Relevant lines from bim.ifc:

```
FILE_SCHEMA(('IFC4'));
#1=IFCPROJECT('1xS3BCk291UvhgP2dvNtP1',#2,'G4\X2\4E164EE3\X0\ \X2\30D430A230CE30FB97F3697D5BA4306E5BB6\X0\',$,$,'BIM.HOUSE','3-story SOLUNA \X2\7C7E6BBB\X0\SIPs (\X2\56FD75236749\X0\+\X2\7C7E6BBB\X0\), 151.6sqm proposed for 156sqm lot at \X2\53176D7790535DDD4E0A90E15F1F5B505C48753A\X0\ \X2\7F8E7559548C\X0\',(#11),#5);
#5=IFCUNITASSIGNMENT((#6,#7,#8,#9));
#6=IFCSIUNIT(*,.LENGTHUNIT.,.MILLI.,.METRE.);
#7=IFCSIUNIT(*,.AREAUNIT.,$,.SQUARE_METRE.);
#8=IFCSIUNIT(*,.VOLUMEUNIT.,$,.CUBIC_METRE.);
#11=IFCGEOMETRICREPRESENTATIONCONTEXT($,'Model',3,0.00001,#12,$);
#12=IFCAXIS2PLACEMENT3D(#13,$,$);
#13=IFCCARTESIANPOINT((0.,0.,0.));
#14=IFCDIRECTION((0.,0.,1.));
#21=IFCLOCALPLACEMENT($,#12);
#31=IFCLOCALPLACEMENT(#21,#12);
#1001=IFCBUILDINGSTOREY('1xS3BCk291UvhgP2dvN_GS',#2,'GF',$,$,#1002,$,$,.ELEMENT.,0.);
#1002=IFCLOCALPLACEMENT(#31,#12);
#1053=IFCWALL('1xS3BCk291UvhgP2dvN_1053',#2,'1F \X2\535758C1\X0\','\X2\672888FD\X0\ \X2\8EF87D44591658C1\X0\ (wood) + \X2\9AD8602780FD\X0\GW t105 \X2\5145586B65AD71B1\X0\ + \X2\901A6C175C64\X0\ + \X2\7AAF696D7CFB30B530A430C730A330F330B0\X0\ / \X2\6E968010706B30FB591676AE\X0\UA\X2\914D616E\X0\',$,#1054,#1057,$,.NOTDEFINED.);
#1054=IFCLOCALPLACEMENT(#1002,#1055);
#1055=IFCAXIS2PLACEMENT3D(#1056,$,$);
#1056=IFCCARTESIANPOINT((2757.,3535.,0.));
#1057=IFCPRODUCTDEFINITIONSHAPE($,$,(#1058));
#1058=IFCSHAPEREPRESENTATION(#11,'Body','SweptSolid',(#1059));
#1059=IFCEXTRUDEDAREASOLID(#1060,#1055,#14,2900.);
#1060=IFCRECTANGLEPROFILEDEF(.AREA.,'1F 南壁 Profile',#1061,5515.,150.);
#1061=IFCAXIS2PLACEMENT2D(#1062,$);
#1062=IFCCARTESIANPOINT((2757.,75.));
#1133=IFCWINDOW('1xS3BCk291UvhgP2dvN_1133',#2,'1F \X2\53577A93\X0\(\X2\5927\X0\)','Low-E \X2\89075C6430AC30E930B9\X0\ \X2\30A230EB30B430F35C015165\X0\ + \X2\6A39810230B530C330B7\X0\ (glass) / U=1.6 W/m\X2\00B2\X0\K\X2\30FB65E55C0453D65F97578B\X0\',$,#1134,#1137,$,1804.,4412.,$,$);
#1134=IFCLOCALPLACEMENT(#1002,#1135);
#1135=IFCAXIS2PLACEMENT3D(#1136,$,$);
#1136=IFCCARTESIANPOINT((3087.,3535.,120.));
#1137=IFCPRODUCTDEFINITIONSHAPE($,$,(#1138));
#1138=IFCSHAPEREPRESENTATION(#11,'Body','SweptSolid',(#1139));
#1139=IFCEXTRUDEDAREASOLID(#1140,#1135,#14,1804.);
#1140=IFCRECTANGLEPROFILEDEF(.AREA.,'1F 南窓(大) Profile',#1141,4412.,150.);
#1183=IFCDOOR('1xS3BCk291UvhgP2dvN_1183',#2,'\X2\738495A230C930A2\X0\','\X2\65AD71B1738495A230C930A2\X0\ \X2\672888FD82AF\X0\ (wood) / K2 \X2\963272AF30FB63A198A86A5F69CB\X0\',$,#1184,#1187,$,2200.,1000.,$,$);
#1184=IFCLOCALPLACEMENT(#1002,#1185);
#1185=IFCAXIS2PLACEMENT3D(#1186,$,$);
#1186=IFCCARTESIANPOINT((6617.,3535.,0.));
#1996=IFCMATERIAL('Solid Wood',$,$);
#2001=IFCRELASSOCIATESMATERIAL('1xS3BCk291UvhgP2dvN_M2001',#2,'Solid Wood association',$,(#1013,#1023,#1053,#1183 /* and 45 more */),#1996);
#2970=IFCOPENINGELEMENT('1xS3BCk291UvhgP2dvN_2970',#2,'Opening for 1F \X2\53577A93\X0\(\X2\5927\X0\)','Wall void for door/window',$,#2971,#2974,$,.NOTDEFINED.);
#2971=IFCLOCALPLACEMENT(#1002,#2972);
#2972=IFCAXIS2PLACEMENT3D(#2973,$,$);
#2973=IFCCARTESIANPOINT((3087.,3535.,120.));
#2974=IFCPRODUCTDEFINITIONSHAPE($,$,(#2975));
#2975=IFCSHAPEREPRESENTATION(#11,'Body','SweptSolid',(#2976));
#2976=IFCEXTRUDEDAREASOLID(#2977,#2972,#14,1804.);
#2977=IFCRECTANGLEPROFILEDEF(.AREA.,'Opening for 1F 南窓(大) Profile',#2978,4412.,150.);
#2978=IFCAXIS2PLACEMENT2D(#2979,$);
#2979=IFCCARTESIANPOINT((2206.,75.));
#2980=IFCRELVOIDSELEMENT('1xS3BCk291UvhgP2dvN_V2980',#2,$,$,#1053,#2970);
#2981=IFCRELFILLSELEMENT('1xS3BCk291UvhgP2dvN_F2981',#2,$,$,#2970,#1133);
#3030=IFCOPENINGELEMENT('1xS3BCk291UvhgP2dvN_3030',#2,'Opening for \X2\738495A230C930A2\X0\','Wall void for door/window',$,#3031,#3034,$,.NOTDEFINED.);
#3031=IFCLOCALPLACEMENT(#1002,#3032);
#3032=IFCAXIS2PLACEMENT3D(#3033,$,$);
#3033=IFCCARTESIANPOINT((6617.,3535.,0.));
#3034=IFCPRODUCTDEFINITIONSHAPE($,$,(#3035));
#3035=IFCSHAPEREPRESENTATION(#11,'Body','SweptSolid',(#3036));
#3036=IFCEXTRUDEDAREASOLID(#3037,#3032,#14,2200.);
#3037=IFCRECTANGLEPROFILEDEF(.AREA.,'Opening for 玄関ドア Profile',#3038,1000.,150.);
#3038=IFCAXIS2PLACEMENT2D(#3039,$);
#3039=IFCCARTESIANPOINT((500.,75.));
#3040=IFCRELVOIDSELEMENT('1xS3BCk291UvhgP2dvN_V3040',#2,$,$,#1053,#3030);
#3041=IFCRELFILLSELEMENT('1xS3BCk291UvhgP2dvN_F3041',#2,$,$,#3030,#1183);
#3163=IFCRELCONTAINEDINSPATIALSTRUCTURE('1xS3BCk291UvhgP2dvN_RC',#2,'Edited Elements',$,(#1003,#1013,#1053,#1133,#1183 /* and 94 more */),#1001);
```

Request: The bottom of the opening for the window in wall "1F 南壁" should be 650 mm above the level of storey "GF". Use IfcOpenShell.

```python
import numpy as np
import ifcopenshell
import ifcopenshell.api.geometry
import ifcopenshell.geom
import ifcopenshell.util.element
import ifcopenshell.util.placement
import ifcopenshell.util.shape
import ifcopenshell.util.unit

model = ifcopenshell.open("bim.ifc")
unit_scale = ifcopenshell.util.unit.calculate_unit_scale(model)

window = model.by_id(1133)
opening = window.FillsVoids[0].RelatingOpeningElement
storey = ifcopenshell.util.element.get_container(window, ifc_class="IfcBuildingStorey")
level = ifcopenshell.util.placement.get_local_placement(storey.ObjectPlacement)[2, 3]

# The opening's origin need not be at the sill, so measure its lowest point.
shape = ifcopenshell.geom.create_shape(ifcopenshell.geom.settings(), opening)
bottom = ifcopenshell.util.shape.get_shape_bottom_elevation(shape, shape.geometry) / unit_scale
dz = level + 650.0 - bottom

shift = np.array([0.0, 0.0, dz])
# The window is not placed relative to its opening, so move both.
for product in (opening, window):
    matrix = ifcopenshell.util.placement.get_local_placement(product.ObjectPlacement)
    matrix[:3, 3] += shift
    ifcopenshell.api.geometry.edit_object_placement(model, product=product, matrix=matrix, is_si=False)

print(f"moved by {dz * unit_scale:+.3f} m")

model.write("bim_updated.ifc")
```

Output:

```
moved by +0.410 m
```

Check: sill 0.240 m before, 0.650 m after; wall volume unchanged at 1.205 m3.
